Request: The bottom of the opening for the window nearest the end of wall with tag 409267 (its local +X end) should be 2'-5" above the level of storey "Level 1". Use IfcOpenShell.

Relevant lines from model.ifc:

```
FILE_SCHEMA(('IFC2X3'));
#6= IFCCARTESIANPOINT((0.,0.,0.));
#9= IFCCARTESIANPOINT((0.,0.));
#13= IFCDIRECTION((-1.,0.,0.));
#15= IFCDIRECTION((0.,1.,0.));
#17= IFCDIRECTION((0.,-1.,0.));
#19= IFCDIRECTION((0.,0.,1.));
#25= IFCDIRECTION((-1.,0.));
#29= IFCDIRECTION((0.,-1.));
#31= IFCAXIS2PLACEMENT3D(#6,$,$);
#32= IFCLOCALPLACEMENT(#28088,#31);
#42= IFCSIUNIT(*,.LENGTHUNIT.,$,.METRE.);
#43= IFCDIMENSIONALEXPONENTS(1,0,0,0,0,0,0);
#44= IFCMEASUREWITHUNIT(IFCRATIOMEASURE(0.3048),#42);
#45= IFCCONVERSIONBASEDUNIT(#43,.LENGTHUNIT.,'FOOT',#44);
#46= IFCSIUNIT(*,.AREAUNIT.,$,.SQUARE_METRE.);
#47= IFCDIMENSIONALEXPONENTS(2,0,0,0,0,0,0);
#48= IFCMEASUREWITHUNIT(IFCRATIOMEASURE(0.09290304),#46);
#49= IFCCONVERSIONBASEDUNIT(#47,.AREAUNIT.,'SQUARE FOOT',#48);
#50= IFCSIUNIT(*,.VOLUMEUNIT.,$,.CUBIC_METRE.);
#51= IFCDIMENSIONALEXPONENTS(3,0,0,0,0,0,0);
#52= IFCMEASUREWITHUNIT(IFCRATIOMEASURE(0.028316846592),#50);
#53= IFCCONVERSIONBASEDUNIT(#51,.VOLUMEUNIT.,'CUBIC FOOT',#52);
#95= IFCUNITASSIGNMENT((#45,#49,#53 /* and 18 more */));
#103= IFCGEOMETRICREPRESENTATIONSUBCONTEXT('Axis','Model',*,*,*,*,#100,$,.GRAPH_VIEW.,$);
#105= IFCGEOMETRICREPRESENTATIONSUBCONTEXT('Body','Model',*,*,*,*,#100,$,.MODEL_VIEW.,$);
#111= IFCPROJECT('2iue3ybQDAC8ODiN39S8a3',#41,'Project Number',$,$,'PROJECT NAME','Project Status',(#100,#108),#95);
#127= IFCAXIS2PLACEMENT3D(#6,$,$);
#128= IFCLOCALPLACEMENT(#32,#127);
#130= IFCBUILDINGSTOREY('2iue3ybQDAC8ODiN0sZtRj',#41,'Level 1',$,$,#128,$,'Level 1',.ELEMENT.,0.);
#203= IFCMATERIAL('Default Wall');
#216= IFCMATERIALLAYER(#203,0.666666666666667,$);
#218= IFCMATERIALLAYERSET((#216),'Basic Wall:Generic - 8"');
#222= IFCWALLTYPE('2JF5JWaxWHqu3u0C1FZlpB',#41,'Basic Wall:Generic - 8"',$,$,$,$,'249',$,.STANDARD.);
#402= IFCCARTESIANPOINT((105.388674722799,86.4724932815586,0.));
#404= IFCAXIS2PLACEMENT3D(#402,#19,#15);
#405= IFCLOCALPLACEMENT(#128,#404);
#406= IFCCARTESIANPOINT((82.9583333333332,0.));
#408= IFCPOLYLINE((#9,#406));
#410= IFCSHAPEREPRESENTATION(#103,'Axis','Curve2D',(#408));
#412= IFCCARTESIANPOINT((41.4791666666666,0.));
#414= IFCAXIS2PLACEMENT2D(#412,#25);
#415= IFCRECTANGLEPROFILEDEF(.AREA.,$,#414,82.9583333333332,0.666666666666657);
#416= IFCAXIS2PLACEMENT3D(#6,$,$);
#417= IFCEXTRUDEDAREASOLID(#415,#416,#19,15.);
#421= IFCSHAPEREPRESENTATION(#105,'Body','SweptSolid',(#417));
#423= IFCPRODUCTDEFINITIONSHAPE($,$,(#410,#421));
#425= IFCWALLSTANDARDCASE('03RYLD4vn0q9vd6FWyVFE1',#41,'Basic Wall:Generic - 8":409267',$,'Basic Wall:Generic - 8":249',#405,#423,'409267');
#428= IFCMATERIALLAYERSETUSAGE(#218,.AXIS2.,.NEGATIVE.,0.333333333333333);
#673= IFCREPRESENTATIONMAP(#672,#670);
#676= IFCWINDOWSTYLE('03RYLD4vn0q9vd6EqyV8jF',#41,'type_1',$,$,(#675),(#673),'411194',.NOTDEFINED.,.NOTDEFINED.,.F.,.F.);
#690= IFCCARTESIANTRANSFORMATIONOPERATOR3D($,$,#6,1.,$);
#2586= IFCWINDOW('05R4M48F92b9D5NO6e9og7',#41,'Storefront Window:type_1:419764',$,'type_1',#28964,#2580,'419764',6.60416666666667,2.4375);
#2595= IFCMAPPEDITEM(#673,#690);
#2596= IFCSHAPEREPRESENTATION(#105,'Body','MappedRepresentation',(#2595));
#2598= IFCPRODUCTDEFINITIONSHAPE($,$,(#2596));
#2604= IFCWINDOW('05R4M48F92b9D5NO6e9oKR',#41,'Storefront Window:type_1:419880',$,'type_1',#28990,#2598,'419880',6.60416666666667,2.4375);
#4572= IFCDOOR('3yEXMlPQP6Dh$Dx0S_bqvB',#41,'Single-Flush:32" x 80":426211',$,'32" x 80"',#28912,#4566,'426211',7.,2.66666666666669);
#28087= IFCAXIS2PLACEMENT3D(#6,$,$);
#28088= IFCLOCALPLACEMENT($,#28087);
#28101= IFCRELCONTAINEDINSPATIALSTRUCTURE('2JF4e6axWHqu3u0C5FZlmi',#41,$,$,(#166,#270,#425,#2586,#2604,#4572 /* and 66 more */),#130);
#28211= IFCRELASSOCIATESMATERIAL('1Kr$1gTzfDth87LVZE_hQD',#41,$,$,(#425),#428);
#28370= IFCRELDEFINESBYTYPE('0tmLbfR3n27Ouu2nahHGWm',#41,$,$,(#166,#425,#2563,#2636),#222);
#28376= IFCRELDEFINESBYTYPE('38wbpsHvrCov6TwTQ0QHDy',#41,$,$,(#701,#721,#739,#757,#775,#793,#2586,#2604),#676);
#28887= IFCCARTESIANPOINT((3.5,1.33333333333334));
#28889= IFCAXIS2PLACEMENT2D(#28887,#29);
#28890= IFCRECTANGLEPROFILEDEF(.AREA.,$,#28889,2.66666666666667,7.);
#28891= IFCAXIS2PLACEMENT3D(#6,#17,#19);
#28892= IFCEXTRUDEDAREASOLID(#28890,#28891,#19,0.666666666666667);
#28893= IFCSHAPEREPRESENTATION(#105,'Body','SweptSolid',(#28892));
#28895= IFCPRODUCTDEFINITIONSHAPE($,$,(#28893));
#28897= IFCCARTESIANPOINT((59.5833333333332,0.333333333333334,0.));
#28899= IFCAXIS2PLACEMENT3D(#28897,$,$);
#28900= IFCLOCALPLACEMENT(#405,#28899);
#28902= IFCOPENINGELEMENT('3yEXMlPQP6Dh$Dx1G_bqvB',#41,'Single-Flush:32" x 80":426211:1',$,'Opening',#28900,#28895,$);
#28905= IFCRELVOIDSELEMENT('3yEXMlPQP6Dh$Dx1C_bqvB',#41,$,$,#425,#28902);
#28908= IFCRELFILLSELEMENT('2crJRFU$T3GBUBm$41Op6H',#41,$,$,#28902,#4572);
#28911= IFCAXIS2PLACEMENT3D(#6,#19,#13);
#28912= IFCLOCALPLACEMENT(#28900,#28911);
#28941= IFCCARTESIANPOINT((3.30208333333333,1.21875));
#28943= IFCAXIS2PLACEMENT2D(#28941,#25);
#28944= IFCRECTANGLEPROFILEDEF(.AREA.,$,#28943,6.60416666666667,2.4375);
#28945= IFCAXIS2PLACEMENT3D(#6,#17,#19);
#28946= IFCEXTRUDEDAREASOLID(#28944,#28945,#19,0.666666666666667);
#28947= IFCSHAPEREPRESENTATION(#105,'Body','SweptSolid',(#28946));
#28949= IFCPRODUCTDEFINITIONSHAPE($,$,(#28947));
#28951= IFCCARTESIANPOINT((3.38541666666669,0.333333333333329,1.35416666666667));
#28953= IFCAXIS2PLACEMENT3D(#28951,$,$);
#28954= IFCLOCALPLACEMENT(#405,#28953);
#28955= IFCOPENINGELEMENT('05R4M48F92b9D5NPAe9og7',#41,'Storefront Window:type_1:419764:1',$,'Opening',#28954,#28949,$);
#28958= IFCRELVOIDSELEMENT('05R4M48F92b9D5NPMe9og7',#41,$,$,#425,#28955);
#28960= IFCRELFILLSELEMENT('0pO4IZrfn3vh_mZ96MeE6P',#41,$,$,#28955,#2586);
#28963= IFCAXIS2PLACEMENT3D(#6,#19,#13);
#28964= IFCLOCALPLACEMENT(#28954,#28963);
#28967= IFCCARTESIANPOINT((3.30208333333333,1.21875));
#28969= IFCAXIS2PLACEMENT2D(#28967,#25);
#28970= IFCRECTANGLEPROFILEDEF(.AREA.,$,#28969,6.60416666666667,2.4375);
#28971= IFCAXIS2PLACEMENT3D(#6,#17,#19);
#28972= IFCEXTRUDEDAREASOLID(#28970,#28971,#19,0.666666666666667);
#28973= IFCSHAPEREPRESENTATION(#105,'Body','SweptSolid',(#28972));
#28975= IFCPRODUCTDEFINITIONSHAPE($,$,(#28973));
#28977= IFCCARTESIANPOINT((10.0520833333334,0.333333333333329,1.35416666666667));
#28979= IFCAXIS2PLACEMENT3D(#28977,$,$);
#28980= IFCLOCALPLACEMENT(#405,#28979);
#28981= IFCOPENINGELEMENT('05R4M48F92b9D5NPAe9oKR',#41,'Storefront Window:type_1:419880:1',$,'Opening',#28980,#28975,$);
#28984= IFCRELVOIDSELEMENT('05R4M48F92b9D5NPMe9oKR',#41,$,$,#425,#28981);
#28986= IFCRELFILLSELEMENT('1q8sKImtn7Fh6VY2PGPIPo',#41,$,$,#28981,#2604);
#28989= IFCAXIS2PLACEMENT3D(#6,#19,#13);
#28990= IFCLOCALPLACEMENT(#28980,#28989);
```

```python
import numpy as np
import ifcopenshell
import ifcopenshell.api.geometry
import ifcopenshell.geom
import ifcopenshell.util.element
import ifcopenshell.util.placement
import ifcopenshell.util.shape
import ifcopenshell.util.unit

model = ifcopenshell.open("model.ifc")
unit_scale = ifcopenshell.util.unit.calculate_unit_scale(model)

window = model.by_guid("05R4M48F92b9D5NO6e9oKR")
opening = window.FillsVoids[0].RelatingOpeningElement
storey = ifcopenshell.util.element.get_container(window, ifc_class="IfcBuildingStorey")
level = ifcopenshell.util.placement.get_local_placement(storey.ObjectPlacement)[2, 3]

# The opening's origin need not be at the sill, so measure its lowest point.
shape = ifcopenshell.geom.create_shape(ifcopenshell.geom.settings(), opening)
bottom = ifcopenshell.util.shape.get_shape_bottom_elevation(shape, shape.geometry) / unit_scale
dz = level + 29 * 0.0254 / unit_scale - bottom

shift = np.array([0.0, 0.0, dz])
# The window is placed relative to its opening, so it follows when the opening moves.
matrix = ifcopenshell.util.placement.get_local_placement(opening.ObjectPlacement)
matrix[:3, 3] += shift
ifcopenshell.api.geometry.edit_object_placement(
    model, product=opening, matrix=matrix, is_si=False, should_transform_children=True
)

print(f"moved by {dz * unit_scale:+.3f} m")

model.write("model_edited.ifc")
```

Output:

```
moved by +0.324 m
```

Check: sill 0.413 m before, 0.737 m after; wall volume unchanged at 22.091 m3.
